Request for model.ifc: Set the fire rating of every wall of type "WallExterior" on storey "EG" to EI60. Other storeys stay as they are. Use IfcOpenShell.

First a look at what the model holds.

```python
import ifcopenshell
import ifcopenshell.util.element

model = ifcopenshell.open("model.ifc")
print(model.schema)
storey = next(s for s in model.by_type("IfcBuildingStorey") if s.Name == "EG")
walls = [e for e in ifcopenshell.util.element.get_decomposition(storey) if e.is_a("IfcWall")]
seen = {}
for e in walls:
    element_type = ifcopenshell.util.element.get_type(e)
    key = (element_type.Name if element_type != e and element_type else None, ifcopenshell.util.element.get_pset(e, "Pset_WallCommon", "FireRating"))
    seen[key] = seen.get(key, 0) + 1
for (name, value), count in sorted(seen.items(), key=str):
    print(count, "x", name, "|", value)
```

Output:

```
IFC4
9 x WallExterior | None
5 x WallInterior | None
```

```python
import ifcopenshell
import ifcopenshell.api.pset
import ifcopenshell.util.element

model = ifcopenshell.open("model.ifc")

storey = next(s for s in model.by_type("IfcBuildingStorey") if s.Name == "EG")
walls = [e for e in ifcopenshell.util.element.get_decomposition(storey) if e.is_a("IfcWall")]

count = 0
for e in walls:
    element_type = ifcopenshell.util.element.get_type(e)
    if element_type in (None, e) or element_type.Name != "WallExterior":
        continue
    # add_pset returns the element's existing set when there is one.
    pset = ifcopenshell.api.pset.add_pset(model, product=e, name="Pset_WallCommon")
    ifcopenshell.api.pset.edit_pset(model, pset=pset, properties={"FireRating": "EI60"})
    count += 1

print(count, "walls updated")

model.write("model_edited.ifc")
```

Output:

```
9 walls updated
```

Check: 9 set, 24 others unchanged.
